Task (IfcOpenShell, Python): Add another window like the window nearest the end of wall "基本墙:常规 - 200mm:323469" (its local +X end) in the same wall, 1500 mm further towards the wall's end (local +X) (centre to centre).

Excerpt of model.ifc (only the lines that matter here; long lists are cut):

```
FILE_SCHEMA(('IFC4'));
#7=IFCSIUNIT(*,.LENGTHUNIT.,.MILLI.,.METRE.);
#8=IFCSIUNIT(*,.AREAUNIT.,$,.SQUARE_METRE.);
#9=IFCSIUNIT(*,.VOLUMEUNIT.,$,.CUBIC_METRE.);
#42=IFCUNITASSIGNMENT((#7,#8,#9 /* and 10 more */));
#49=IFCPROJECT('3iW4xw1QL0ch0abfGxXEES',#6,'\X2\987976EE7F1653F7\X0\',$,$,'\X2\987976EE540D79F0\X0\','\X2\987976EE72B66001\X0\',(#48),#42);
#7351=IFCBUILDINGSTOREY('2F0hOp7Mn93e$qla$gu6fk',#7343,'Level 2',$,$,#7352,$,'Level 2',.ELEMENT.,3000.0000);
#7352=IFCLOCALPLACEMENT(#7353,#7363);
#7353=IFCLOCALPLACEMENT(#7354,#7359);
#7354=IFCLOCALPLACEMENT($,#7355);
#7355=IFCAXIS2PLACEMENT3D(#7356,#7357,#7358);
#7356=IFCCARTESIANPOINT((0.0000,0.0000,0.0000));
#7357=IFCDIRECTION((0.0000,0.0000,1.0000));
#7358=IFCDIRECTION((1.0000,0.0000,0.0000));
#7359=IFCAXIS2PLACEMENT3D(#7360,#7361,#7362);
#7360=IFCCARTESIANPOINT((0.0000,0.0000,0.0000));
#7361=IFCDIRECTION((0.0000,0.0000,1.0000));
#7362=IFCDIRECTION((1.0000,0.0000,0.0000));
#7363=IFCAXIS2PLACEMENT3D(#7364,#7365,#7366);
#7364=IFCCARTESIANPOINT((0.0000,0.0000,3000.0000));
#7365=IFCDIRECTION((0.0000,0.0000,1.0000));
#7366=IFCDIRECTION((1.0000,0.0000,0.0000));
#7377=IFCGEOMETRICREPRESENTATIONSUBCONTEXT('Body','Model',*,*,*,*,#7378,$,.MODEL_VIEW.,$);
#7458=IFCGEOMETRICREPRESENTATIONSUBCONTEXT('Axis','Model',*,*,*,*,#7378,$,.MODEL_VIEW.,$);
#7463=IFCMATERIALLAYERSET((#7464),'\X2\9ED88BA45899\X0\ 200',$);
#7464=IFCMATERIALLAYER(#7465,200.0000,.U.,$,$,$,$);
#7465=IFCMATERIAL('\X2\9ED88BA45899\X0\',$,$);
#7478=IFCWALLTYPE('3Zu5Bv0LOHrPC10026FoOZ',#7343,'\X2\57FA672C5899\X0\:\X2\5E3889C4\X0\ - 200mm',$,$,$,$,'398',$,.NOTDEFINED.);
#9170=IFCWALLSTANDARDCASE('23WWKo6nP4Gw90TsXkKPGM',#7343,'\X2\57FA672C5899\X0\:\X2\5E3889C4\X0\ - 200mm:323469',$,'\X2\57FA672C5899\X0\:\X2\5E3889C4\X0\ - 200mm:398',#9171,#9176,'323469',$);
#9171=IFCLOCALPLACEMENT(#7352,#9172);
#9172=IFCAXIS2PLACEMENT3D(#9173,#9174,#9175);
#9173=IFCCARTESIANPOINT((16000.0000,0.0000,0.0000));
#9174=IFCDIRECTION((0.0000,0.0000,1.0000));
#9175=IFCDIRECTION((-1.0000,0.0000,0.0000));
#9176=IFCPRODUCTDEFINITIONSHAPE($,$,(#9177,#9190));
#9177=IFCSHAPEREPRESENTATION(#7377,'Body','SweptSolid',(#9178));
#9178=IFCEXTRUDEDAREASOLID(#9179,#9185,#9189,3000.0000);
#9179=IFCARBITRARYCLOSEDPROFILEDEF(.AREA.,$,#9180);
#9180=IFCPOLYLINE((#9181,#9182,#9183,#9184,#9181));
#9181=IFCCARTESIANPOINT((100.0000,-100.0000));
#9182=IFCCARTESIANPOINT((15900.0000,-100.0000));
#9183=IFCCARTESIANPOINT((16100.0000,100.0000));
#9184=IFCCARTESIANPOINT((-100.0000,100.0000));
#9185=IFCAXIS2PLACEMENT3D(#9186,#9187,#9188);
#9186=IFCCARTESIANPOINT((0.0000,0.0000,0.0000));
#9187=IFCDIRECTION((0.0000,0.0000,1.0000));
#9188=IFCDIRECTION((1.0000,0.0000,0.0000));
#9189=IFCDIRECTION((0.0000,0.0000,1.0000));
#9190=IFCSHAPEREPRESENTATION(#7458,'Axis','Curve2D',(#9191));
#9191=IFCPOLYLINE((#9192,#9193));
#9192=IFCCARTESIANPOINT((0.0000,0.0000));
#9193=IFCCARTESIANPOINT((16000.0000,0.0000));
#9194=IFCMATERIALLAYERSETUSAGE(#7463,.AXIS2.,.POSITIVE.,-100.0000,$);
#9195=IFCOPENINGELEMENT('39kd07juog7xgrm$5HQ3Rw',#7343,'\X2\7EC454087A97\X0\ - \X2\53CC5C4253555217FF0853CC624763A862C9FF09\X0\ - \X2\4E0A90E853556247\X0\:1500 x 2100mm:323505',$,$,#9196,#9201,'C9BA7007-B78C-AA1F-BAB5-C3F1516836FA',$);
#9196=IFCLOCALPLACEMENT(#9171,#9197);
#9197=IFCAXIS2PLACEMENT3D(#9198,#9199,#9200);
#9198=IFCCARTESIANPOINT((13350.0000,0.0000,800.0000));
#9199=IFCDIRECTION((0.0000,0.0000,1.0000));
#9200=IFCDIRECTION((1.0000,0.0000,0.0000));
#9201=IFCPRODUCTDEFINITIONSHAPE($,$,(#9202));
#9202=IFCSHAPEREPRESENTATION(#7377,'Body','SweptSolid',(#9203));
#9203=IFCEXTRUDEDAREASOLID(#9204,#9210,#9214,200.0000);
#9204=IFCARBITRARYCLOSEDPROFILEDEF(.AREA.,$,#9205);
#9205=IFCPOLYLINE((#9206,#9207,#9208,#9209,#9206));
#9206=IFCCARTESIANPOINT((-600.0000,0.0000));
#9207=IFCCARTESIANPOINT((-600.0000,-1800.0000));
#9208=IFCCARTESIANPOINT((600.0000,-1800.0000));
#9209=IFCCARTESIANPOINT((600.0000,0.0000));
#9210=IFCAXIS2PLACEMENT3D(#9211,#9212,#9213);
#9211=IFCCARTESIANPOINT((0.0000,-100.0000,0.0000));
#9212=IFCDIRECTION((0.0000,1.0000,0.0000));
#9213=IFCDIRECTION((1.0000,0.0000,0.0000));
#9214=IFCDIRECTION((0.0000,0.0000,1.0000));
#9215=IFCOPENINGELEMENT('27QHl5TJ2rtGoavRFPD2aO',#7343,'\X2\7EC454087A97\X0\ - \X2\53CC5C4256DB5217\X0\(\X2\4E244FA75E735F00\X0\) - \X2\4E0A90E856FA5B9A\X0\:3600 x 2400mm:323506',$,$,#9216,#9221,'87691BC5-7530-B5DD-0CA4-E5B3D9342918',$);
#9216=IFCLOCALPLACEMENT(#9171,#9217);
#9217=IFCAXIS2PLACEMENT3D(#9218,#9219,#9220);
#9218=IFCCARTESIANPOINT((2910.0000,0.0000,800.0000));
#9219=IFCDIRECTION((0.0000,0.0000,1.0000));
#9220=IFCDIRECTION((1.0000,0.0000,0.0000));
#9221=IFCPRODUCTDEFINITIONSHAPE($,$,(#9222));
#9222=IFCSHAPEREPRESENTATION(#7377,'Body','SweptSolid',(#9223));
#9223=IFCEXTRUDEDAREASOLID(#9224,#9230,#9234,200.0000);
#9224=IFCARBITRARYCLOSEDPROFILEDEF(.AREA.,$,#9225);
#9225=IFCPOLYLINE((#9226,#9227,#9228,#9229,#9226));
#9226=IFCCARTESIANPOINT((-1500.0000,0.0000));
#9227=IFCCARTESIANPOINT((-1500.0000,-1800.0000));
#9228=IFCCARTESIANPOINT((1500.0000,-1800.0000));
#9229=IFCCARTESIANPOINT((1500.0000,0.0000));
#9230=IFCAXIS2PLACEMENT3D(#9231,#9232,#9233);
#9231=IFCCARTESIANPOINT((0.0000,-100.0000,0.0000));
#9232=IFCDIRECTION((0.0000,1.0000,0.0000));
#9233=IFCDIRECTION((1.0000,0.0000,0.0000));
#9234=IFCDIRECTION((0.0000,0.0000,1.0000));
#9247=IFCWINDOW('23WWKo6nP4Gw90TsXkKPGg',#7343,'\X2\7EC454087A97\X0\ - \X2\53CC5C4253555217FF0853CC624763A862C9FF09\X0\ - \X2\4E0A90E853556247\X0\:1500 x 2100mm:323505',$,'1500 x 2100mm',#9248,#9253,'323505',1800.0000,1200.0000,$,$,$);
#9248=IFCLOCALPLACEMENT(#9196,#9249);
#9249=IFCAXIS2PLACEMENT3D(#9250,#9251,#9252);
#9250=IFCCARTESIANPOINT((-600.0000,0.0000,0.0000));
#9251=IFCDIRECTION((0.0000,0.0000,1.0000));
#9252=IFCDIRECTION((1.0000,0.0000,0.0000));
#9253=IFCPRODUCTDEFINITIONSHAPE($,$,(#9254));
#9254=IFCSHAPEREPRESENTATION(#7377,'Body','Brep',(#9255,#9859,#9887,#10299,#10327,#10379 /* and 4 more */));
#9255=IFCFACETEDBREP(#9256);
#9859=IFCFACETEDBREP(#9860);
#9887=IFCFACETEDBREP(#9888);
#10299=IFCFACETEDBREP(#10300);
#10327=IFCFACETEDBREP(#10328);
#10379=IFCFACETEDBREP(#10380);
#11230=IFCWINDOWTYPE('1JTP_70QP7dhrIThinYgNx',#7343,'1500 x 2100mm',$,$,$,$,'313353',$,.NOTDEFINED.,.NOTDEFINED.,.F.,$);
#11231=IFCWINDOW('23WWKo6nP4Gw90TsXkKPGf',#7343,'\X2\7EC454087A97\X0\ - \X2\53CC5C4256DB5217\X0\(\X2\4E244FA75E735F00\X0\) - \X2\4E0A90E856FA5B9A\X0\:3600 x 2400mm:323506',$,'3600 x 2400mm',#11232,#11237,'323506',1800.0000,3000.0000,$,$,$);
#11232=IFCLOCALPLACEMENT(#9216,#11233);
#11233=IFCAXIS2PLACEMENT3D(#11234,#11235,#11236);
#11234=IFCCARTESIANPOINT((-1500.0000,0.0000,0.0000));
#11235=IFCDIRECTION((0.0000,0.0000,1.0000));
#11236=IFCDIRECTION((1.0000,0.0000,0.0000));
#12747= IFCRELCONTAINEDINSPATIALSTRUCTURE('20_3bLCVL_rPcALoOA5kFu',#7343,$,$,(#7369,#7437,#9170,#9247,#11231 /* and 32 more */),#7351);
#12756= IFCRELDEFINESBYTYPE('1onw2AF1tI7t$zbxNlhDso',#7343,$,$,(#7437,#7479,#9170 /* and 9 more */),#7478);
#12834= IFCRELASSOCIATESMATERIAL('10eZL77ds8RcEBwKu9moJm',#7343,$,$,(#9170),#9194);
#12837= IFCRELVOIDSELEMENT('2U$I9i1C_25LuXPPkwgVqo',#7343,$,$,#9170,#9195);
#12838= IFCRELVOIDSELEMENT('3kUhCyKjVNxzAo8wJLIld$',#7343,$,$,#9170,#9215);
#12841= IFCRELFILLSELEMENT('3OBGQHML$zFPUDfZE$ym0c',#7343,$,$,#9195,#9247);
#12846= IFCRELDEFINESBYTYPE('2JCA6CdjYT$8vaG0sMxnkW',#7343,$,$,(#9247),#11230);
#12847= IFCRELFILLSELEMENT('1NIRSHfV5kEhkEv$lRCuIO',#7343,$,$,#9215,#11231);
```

```python
import ifcopenshell
import ifcopenshell.api.feature
import ifcopenshell.api.geometry
import ifcopenshell.api.root
import ifcopenshell.geom
import ifcopenshell.util.element
import ifcopenshell.util.placement
import ifcopenshell.util.shape
import ifcopenshell.util.unit

model = ifcopenshell.open("model.ifc")
unit_scale = ifcopenshell.util.unit.calculate_unit_scale(model)
settings = ifcopenshell.geom.settings()


def volume(element):
    """Net volume in cubic metres, openings subtracted."""
    shape = ifcopenshell.geom.create_shape(settings, element)
    return ifcopenshell.util.shape.get_volume(shape.geometry)


def reuse_history(source, copy):
    """copy_class also copies each property set's owner history, people and application; keep the originals."""
    for rel in copy.IsDefinedBy:
        if rel.is_a("IfcRelDefinesByProperties") and (history := rel.RelatingPropertyDefinition.OwnerHistory):
            rel.RelatingPropertyDefinition.OwnerHistory = source.OwnerHistory
            ifcopenshell.util.element.remove_deep2(model, history)


window = model.by_guid("23WWKo6nP4Gw90TsXkKPGg")
opening = window.FillsVoids[0].RelatingOpeningElement
wall = opening.VoidsElements[0].RelatingBuildingElement
before = volume(wall)
shift = ifcopenshell.util.placement.get_local_placement(wall.ObjectPlacement)[:3, 0] * 1.5 / unit_scale

# copy_class copies the void relationship, type, container and properties, but no geometry.
new_opening = ifcopenshell.api.root.copy_class(model, product=opening)
new_opening.Representation = ifcopenshell.util.element.copy_deep(
    model, opening.Representation, exclude=["IfcGeometricRepresentationContext", "IfcRepresentationMap"]
)
new_opening.Name = "组合窗 - 双层单列（双扇推拉） - 上部单扇:1500 x 2100mm"
new_opening.Tag = None
new_window = ifcopenshell.api.root.copy_class(model, product=window)
new_window.Representation = ifcopenshell.util.element.copy_deep(
    model, window.Representation, exclude=["IfcGeometricRepresentationContext", "IfcRepresentationMap"]
)
new_window.Name = "组合窗 - 双层单列（双扇推拉） - 上部单扇:1500 x 2100mm"
new_window.Tag = None
reuse_history(window, new_window)
ifcopenshell.api.feature.add_filling(model, opening=new_opening, element=new_window)

for old, new in ((opening, new_opening), (window, new_window)):
    matrix = ifcopenshell.util.placement.get_local_placement(old.ObjectPlacement)
    matrix[:3, 3] += shift
    ifcopenshell.api.geometry.edit_object_placement(model, product=new, matrix=matrix, is_si=False)

after = volume(wall)

print(f"wall volume {before:.3f} -> {after:.3f} m3")

model.write("model_v2.ifc")
```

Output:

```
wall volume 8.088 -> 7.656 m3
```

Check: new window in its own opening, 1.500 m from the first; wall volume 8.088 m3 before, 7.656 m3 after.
